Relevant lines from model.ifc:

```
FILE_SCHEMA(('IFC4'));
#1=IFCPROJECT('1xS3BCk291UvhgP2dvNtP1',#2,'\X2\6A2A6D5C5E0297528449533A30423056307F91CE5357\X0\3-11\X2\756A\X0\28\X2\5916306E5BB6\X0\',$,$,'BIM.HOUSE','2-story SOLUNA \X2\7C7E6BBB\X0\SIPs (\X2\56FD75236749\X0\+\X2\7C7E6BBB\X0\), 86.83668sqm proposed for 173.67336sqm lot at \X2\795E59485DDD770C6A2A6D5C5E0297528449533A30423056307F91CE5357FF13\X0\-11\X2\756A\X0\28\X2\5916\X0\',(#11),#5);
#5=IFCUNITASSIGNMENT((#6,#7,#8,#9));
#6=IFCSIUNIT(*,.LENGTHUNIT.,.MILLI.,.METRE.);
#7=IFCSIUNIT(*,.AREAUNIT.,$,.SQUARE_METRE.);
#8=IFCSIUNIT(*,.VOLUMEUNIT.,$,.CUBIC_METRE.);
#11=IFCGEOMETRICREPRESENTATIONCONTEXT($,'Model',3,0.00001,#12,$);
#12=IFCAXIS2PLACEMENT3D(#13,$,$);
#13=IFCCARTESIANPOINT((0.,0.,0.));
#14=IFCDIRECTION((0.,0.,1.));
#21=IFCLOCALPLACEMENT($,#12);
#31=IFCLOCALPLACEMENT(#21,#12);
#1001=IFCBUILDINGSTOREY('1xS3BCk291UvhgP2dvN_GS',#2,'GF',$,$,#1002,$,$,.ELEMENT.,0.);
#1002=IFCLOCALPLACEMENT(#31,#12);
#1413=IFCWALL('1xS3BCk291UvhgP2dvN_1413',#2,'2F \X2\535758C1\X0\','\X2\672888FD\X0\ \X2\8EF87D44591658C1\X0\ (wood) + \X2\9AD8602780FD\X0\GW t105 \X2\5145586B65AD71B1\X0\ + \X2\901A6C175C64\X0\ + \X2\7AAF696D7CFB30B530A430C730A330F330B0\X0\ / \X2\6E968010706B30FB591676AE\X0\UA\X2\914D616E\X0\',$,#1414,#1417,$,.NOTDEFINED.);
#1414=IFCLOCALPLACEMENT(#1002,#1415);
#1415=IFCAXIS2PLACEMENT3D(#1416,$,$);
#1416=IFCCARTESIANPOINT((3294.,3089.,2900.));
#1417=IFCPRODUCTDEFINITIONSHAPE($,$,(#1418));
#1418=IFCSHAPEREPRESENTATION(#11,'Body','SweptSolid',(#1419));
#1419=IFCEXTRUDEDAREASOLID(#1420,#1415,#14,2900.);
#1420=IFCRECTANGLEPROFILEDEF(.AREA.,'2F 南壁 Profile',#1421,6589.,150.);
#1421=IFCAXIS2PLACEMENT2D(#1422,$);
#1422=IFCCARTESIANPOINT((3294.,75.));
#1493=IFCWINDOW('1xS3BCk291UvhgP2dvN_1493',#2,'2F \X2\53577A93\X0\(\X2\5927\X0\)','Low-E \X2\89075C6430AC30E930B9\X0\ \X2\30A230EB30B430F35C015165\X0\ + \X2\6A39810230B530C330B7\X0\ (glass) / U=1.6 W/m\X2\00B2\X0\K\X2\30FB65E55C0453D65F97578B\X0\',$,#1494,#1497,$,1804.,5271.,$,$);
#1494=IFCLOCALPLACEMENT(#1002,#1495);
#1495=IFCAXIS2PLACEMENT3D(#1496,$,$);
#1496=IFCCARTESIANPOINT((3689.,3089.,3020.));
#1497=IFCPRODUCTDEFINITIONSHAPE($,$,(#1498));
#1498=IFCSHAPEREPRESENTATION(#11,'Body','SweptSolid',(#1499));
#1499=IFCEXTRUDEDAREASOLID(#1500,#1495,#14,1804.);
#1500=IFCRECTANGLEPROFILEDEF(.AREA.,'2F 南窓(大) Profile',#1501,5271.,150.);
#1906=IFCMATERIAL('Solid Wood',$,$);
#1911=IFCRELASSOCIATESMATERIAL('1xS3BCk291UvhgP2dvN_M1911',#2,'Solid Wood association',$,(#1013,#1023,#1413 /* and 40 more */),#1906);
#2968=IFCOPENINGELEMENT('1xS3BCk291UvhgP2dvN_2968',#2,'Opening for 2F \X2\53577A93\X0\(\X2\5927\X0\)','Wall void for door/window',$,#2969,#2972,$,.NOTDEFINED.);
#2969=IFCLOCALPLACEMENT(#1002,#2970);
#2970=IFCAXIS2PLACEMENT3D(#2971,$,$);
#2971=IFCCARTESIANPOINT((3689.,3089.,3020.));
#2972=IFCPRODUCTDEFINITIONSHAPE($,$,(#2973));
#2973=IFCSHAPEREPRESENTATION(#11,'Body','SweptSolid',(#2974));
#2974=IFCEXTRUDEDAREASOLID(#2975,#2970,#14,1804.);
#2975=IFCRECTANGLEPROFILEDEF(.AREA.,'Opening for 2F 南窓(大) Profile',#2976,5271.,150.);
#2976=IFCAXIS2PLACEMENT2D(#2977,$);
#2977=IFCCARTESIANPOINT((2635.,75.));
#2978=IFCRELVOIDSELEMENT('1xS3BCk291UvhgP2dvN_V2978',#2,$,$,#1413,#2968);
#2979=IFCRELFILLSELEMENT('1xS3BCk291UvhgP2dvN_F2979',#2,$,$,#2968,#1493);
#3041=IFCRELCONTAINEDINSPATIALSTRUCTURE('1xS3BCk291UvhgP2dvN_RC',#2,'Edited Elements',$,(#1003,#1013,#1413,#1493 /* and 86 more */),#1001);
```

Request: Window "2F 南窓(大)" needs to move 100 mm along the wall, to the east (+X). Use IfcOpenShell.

```python
import ifcopenshell
import ifcopenshell.api.geometry
import ifcopenshell.util.placement

model = ifcopenshell.open("model.ifc")

window = model.by_id(1493)
opening = window.FillsVoids[0].RelatingOpeningElement
wall = opening.VoidsElements[0].RelatingBuildingElement

wall_matrix = ifcopenshell.util.placement.get_local_placement(wall.ObjectPlacement)
shift = wall_matrix[:3, 0] * 100.0
before = ifcopenshell.util.placement.get_local_placement(window.ObjectPlacement)[:3, 3].copy()

# The window is not placed relative to its opening, so move both.
for product in (opening, window):
    matrix = ifcopenshell.util.placement.get_local_placement(product.ObjectPlacement)
    matrix[:3, 3] += shift
    ifcopenshell.api.geometry.edit_object_placement(model, product=product, matrix=matrix, is_si=False)

after = ifcopenshell.util.placement.get_local_placement(window.ObjectPlacement)[:3, 3]
print("window moved by", (after - before).round(3) + 0.0)

model.write("model_rev.ifc")
```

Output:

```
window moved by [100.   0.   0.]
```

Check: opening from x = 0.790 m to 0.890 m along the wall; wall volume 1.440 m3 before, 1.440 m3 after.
